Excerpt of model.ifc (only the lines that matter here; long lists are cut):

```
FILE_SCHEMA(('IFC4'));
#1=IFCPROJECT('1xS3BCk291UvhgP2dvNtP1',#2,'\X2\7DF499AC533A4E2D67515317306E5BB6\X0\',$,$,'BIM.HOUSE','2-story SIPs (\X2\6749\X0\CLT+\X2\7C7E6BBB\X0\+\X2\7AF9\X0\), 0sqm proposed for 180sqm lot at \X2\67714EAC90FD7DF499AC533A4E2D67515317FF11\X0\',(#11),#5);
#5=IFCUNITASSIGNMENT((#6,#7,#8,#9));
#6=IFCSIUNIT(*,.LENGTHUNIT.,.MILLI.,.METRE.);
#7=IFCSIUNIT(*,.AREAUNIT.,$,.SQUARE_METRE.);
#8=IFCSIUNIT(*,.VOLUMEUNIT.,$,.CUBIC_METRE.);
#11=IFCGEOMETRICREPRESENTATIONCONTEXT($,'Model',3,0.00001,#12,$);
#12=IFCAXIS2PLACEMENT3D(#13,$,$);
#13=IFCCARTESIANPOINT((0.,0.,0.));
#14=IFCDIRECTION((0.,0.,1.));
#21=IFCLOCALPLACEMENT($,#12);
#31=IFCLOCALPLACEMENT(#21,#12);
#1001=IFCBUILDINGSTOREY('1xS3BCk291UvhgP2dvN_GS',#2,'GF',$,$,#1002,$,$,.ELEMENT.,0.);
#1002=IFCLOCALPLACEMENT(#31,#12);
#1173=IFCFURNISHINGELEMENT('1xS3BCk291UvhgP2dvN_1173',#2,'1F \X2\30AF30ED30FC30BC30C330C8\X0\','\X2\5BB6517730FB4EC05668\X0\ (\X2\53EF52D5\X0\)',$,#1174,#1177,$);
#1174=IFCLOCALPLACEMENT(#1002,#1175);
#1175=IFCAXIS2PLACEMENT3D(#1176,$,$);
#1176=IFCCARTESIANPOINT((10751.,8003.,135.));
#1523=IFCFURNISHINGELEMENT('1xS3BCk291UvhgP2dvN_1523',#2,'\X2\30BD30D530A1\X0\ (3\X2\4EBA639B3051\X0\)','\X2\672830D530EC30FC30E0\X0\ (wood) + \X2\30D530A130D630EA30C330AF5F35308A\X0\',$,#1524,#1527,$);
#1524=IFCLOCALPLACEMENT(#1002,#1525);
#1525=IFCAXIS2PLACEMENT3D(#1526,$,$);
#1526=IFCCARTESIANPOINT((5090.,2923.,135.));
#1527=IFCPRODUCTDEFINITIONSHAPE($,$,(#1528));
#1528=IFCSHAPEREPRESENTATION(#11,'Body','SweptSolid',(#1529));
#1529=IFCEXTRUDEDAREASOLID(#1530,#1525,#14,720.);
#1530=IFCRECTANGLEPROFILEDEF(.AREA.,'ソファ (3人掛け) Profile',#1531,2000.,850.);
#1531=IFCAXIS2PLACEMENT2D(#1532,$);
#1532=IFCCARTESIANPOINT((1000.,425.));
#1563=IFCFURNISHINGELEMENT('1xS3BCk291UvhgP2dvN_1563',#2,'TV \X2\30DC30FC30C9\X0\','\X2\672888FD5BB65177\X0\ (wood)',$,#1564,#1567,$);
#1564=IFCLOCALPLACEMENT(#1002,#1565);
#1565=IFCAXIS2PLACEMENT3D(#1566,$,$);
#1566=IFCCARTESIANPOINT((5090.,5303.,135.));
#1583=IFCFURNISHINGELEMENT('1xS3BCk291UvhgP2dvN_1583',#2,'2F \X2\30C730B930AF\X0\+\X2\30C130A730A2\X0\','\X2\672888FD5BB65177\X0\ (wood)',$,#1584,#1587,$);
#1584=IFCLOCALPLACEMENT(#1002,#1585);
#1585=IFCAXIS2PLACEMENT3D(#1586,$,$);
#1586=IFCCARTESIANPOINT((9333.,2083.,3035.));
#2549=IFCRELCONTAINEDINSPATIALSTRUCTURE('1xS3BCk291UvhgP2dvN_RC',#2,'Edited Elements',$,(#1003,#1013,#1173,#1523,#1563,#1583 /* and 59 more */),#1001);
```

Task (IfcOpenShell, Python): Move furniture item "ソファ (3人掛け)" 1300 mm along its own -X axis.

```python
import ifcopenshell
import ifcopenshell.api.geometry
import ifcopenshell.util.placement

model = ifcopenshell.open("model.ifc")

item = model.by_id(1523)
matrix = ifcopenshell.util.placement.get_local_placement(item.ObjectPlacement)
matrix[:3, 3] -= matrix[:3, 0] * 1300.0
ifcopenshell.api.geometry.edit_object_placement(model, product=item, matrix=matrix, is_si=False)

print(ifcopenshell.util.placement.get_local_placement(item.ObjectPlacement).round(3) + 0.0)

model.write("model-out.ifc")
```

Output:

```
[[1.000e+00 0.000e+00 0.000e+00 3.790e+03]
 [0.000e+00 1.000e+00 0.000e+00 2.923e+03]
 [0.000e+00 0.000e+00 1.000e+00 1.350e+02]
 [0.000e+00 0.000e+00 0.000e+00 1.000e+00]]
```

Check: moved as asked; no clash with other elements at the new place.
